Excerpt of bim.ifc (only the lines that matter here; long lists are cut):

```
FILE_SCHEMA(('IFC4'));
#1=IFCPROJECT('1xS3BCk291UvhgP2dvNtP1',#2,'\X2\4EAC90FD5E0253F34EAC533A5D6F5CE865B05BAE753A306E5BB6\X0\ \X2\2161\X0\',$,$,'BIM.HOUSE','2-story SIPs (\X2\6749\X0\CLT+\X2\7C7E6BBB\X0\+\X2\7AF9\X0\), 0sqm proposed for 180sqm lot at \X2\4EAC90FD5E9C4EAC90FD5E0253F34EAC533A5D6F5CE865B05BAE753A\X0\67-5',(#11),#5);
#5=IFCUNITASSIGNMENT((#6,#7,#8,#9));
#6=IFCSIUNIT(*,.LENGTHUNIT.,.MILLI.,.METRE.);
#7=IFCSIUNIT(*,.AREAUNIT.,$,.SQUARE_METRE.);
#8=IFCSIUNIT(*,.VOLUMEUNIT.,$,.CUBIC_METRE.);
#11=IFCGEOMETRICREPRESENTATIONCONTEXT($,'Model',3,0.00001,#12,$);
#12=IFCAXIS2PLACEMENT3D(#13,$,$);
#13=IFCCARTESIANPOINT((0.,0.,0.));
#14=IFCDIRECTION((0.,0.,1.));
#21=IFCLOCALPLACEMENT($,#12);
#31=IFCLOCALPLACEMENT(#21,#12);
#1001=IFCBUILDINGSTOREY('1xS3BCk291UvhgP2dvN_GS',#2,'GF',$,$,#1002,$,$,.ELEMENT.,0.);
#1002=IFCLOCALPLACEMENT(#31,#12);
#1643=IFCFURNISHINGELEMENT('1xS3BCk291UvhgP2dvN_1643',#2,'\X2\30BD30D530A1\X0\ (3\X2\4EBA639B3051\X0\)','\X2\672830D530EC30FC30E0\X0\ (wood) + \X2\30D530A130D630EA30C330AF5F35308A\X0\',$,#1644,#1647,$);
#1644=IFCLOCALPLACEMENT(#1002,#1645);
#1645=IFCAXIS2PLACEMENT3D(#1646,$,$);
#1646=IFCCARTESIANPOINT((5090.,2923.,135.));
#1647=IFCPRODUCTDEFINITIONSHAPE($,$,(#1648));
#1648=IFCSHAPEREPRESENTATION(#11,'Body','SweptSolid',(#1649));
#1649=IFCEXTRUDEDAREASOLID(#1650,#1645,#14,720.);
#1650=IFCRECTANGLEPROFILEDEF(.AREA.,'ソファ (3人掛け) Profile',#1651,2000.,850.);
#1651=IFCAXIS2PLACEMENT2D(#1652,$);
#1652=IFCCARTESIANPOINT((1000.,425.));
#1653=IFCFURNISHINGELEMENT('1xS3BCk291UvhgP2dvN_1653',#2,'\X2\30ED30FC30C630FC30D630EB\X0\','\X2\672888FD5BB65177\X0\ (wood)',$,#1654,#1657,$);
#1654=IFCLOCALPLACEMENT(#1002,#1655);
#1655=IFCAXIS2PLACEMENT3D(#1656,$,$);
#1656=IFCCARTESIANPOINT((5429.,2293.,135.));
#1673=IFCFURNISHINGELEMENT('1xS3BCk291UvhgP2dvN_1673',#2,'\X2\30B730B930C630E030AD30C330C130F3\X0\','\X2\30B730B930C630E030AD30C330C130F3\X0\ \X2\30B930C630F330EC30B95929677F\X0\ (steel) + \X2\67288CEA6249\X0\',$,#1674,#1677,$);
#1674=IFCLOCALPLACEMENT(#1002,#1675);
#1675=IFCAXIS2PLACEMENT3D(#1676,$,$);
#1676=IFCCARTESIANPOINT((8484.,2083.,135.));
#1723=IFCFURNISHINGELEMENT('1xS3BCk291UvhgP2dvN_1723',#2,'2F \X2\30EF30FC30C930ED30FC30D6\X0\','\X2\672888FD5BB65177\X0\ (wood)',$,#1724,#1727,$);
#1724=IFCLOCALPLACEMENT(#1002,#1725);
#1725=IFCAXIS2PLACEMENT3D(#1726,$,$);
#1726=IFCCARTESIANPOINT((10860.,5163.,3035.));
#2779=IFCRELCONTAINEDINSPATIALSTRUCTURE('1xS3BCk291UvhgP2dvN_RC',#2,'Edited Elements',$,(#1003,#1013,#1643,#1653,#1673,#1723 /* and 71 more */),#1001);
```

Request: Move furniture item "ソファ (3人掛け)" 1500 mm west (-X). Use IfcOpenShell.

```python
import ifcopenshell
import ifcopenshell.api.geometry
import ifcopenshell.util.placement

model = ifcopenshell.open("bim.ifc")

item = model.by_guid("1xS3BCk291UvhgP2dvN_1643")
matrix = ifcopenshell.util.placement.get_local_placement(item.ObjectPlacement)
matrix[0, 3] -= 1500.0
ifcopenshell.api.geometry.edit_object_placement(model, product=item, matrix=matrix, is_si=False)

print(ifcopenshell.util.placement.get_local_placement(item.ObjectPlacement).round(3) + 0.0)

model.write("bim-out.ifc")
```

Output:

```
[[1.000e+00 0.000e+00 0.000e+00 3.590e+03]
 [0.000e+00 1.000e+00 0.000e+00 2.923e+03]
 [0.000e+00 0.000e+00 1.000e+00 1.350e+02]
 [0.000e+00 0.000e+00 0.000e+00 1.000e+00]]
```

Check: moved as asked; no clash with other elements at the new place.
